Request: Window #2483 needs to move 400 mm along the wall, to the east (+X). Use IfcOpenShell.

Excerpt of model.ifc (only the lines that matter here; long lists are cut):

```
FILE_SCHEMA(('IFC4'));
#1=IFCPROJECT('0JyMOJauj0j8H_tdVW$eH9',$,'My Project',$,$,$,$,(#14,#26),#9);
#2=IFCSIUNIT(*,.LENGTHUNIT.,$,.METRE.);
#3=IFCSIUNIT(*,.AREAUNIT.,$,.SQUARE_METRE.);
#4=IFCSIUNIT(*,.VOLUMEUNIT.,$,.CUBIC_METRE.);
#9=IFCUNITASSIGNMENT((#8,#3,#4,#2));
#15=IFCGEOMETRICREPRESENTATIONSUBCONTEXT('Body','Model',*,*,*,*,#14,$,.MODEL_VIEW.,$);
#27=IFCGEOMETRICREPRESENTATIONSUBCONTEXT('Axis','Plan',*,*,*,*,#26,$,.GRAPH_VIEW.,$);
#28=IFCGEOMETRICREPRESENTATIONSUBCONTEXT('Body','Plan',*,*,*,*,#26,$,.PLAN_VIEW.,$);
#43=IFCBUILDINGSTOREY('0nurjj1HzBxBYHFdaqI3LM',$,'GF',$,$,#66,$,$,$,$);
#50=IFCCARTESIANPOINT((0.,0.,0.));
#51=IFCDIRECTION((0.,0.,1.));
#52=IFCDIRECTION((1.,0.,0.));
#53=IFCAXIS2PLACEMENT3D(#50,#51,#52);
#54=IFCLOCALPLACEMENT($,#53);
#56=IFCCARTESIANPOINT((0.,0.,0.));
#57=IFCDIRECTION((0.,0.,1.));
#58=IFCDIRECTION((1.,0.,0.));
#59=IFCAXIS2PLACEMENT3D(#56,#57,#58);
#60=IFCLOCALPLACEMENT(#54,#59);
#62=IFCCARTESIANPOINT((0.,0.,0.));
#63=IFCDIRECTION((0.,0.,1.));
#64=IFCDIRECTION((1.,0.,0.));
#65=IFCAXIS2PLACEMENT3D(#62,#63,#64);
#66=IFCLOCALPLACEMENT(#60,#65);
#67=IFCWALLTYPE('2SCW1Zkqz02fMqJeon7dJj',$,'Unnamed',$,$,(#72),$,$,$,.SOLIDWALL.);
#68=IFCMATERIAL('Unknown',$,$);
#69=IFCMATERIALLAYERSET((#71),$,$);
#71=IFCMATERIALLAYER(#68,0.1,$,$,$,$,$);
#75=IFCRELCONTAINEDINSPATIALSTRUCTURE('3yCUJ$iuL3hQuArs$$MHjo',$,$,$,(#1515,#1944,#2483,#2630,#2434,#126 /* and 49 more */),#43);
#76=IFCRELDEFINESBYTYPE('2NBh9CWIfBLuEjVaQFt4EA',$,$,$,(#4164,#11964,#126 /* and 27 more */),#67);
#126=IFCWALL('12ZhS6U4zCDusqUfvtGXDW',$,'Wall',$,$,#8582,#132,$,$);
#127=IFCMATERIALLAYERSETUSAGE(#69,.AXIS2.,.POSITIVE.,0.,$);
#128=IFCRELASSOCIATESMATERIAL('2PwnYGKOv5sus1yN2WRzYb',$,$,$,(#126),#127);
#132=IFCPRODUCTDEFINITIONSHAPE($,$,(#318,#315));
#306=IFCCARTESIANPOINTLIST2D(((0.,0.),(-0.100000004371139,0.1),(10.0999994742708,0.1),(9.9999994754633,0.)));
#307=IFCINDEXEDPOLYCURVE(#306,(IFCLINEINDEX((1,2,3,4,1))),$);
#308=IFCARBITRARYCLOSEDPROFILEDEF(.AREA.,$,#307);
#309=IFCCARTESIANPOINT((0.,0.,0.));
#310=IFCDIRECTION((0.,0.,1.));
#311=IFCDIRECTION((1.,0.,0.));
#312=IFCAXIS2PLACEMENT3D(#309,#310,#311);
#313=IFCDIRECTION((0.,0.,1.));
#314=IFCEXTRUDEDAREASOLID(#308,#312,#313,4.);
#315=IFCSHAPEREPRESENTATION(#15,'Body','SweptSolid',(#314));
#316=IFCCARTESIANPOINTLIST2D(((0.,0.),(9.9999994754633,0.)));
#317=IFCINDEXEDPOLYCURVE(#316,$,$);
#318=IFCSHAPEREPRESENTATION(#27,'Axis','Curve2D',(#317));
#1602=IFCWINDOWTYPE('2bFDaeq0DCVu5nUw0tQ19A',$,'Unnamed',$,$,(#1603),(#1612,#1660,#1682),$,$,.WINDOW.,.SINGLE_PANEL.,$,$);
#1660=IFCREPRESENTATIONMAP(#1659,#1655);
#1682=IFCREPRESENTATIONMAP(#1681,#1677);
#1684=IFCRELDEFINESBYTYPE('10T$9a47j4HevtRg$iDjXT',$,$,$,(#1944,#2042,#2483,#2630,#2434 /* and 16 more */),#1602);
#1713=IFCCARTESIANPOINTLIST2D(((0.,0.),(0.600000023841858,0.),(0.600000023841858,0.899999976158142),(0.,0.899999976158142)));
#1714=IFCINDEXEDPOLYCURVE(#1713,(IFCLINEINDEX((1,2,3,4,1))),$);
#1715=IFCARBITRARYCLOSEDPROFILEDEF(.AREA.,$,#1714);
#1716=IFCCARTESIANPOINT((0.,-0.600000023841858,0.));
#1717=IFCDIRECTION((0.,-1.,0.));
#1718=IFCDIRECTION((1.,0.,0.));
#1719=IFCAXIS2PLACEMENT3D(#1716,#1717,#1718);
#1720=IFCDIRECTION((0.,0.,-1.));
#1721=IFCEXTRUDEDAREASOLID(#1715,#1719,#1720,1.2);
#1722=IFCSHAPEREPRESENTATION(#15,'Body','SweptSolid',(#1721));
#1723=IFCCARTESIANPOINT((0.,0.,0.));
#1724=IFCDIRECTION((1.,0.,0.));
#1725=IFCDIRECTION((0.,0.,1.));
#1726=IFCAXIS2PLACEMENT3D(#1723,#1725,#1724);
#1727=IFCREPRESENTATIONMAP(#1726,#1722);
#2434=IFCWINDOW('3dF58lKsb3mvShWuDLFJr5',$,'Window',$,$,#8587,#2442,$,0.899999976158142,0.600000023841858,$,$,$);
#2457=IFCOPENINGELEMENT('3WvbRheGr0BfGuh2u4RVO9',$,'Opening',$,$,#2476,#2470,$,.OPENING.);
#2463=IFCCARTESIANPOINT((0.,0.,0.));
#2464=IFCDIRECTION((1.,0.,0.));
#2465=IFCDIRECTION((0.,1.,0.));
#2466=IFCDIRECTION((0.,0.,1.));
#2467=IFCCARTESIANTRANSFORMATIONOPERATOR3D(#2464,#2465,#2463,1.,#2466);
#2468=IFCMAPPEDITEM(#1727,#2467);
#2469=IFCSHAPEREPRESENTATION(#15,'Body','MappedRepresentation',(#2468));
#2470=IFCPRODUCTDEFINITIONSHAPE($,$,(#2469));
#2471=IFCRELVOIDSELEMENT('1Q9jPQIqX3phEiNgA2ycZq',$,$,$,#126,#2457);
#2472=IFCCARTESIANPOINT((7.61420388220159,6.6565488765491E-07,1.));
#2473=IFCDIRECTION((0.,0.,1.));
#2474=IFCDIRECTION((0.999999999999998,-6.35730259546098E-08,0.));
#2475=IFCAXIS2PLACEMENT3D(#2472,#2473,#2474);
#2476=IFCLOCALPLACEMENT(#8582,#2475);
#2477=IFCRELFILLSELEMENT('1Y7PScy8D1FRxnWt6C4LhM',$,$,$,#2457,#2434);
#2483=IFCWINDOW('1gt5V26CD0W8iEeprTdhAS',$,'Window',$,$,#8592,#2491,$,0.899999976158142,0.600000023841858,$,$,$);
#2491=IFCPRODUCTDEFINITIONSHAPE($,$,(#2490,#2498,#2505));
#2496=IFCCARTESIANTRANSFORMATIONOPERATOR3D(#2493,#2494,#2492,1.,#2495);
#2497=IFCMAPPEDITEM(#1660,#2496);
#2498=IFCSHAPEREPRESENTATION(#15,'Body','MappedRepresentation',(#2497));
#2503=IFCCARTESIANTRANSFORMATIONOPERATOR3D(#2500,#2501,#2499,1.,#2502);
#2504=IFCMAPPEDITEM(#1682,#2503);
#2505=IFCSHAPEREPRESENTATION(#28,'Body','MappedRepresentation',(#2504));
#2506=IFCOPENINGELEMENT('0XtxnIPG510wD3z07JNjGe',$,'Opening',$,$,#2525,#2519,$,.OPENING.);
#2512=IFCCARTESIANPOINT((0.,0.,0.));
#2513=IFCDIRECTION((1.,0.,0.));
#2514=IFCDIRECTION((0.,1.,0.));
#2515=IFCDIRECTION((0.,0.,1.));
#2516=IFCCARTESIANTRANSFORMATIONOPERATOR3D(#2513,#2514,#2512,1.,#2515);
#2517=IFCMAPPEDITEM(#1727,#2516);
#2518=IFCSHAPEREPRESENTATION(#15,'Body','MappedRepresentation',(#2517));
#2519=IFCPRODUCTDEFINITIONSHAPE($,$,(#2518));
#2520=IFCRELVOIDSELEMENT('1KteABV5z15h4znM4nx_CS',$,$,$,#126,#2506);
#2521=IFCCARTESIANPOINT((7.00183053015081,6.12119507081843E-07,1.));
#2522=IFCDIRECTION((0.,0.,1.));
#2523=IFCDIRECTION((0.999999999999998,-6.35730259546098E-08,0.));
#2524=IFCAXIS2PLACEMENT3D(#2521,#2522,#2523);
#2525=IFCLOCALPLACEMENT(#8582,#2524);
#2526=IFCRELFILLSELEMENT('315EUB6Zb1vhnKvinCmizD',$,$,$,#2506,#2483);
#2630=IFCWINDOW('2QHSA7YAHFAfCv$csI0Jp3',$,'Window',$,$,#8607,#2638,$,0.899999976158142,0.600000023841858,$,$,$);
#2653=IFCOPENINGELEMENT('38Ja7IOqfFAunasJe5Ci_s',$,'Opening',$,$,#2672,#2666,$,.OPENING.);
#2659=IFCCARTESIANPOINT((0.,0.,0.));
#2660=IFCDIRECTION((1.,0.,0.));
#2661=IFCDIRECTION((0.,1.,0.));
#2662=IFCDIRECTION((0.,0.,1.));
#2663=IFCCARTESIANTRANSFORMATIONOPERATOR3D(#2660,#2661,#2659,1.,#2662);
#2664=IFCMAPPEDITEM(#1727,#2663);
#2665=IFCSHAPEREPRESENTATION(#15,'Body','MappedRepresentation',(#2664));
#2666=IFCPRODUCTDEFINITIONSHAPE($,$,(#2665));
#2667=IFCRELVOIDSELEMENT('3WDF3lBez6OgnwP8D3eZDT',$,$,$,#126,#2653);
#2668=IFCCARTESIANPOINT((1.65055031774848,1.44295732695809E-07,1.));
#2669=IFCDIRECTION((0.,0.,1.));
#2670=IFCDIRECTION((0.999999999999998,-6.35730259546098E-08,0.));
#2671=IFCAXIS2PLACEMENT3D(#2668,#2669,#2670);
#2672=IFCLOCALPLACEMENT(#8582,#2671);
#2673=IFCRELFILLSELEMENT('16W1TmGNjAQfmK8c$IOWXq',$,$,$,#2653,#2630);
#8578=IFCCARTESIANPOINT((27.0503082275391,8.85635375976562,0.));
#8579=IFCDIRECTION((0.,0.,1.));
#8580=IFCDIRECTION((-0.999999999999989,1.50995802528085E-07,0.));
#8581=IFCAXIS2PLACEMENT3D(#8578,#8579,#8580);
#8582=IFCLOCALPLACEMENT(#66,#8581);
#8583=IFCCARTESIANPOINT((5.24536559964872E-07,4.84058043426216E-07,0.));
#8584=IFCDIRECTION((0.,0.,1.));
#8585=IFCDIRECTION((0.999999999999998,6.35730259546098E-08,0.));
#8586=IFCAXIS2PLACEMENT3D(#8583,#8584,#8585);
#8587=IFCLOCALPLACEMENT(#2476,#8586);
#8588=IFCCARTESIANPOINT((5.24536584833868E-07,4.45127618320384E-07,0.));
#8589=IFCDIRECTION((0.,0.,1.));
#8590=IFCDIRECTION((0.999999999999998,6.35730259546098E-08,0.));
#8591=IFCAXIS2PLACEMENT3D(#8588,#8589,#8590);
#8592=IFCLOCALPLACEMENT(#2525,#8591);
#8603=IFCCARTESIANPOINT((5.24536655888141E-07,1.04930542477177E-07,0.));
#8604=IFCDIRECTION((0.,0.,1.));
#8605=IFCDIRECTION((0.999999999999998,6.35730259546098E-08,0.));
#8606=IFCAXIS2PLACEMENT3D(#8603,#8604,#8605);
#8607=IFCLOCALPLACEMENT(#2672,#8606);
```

```python
import ifcopenshell
import ifcopenshell.api.geometry
import ifcopenshell.util.placement

model = ifcopenshell.open("model.ifc")

window = model.by_id(2483)
opening = window.FillsVoids[0].RelatingOpeningElement
wall = opening.VoidsElements[0].RelatingBuildingElement

wall_matrix = ifcopenshell.util.placement.get_local_placement(wall.ObjectPlacement)
shift = wall_matrix[:3, 0] * -0.4
before = ifcopenshell.util.placement.get_local_placement(window.ObjectPlacement)[:3, 3].copy()

# The window is placed relative to its opening, so it follows when the opening moves.
matrix = ifcopenshell.util.placement.get_local_placement(opening.ObjectPlacement)
matrix[:3, 3] += shift
ifcopenshell.api.geometry.edit_object_placement(
    model, product=opening, matrix=matrix, is_si=False, should_transform_children=True
)

after = ifcopenshell.util.placement.get_local_placement(window.ObjectPlacement)[:3, 3]
print("window moved by", (after - before).round(3) + 0.0)

model.write("model_updated.ifc")
```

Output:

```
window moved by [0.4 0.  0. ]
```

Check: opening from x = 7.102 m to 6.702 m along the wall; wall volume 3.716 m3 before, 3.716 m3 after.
